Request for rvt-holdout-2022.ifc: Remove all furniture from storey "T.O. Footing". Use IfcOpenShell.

First a look at what the model holds.

```python
import ifcopenshell
import ifcopenshell.util.element

model = ifcopenshell.open("rvt-holdout-2022.ifc")
print(model.schema)
storey = next(s for s in model.by_type("IfcBuildingStorey") if s.Name == "T.O. Footing")
furniture = [e for e in ifcopenshell.util.element.get_decomposition(storey) if e.is_a("IfcFurnishingElement")]
seen = {}
for e in furniture:
    element_type = ifcopenshell.util.element.get_type(e)
    name = element_type.Name if element_type not in (None, e) else None
    seen[name] = seen.get(name, 0) + 1
for name, count in sorted(seen.items(), key=str):
    print(count, "x", name)
```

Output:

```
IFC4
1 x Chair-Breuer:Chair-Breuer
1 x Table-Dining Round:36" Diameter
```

```python
import ifcopenshell
import ifcopenshell.api.root
import ifcopenshell.util.element

model = ifcopenshell.open("rvt-holdout-2022.ifc")

storey = next(s for s in model.by_type("IfcBuildingStorey") if s.Name == "T.O. Footing")
furniture = [e for e in ifcopenshell.util.element.get_decomposition(storey) if e.is_a("IfcFurnishingElement")]

for e in furniture:
    ifcopenshell.api.root.remove_product(model, product=e)
print(len(furniture), "removed")

model.write("rvt-holdout-2022_rev.ifc")
```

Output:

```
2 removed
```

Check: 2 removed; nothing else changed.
